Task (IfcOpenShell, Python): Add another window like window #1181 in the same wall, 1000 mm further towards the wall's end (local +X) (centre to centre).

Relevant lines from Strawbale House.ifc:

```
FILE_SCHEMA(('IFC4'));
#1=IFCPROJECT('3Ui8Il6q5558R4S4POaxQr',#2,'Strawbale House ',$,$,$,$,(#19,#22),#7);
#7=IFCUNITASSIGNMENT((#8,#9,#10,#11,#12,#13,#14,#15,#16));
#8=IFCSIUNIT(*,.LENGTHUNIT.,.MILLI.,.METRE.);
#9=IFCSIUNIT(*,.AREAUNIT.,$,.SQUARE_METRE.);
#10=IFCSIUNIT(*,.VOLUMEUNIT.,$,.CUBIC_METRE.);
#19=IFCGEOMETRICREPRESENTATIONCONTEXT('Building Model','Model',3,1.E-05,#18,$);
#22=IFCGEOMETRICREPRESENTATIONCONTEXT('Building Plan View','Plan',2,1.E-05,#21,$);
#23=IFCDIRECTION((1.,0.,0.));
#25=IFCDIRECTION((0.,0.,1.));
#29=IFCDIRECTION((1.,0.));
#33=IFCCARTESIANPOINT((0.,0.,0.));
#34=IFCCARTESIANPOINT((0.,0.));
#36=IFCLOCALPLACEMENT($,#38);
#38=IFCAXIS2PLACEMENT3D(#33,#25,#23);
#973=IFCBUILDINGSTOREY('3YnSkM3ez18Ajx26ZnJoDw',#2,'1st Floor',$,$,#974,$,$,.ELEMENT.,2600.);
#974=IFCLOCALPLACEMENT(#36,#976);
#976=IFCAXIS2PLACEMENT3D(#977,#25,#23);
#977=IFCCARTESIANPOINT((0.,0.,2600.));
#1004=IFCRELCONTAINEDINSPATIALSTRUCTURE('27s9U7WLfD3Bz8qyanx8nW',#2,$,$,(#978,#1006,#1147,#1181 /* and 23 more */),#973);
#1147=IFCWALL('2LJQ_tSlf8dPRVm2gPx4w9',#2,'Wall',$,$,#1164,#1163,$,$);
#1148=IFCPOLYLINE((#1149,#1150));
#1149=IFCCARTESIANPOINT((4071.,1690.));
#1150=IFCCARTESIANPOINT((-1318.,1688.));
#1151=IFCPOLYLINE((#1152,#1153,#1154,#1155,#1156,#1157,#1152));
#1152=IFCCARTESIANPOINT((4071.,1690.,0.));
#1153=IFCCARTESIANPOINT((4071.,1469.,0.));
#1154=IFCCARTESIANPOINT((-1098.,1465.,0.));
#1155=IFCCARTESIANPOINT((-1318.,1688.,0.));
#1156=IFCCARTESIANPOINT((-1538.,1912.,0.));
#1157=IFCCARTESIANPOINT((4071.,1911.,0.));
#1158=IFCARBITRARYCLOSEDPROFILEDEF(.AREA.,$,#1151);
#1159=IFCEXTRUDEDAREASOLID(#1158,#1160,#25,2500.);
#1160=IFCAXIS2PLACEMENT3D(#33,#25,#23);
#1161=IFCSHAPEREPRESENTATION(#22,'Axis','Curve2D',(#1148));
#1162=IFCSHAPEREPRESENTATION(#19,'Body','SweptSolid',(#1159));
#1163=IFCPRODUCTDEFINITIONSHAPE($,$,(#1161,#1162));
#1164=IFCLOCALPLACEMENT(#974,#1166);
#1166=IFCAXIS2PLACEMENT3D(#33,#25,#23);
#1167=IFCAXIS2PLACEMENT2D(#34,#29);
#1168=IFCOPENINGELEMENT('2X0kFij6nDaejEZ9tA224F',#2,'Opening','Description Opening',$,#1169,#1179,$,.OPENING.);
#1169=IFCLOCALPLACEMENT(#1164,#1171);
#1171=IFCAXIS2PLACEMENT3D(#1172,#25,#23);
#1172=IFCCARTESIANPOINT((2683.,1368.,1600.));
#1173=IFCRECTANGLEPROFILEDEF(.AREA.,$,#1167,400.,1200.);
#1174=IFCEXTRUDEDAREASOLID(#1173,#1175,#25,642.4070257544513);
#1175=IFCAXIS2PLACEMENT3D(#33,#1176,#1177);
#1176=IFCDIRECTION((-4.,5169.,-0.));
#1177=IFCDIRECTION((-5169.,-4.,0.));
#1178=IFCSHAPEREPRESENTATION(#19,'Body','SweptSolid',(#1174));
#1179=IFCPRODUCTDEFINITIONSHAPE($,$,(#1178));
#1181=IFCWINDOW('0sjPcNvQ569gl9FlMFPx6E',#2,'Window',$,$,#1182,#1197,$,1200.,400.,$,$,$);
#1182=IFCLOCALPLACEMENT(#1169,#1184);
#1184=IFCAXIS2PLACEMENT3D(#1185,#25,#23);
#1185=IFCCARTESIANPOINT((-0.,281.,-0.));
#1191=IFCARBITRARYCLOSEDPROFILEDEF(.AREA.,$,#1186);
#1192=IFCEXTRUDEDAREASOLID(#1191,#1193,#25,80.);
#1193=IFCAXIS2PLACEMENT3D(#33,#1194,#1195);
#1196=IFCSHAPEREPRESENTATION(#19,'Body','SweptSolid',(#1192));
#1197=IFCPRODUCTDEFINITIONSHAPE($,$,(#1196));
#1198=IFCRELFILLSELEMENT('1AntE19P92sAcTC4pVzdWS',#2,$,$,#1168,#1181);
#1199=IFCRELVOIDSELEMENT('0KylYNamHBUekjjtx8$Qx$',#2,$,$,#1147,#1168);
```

```python
import ifcopenshell
import ifcopenshell.api.feature
import ifcopenshell.api.geometry
import ifcopenshell.api.root
import ifcopenshell.geom
import ifcopenshell.util.element
import ifcopenshell.util.placement
import ifcopenshell.util.shape
import ifcopenshell.util.unit

model = ifcopenshell.open("Strawbale House.ifc")
unit_scale = ifcopenshell.util.unit.calculate_unit_scale(model)
settings = ifcopenshell.geom.settings()


def volume(element):
    """Net volume in cubic metres, openings subtracted."""
    shape = ifcopenshell.geom.create_shape(settings, element)
    return ifcopenshell.util.shape.get_volume(shape.geometry)


window = model.by_guid("0sjPcNvQ569gl9FlMFPx6E")
opening = window.FillsVoids[0].RelatingOpeningElement
wall = opening.VoidsElements[0].RelatingBuildingElement
before = volume(wall)
shift = ifcopenshell.util.placement.get_local_placement(wall.ObjectPlacement)[:3, 0] * 1 / unit_scale

# copy_class copies the void relationship, type, container and properties, but no geometry.
new_opening = ifcopenshell.api.root.copy_class(model, product=opening)
new_opening.Representation = ifcopenshell.util.element.copy_deep(
    model, opening.Representation, exclude=["IfcGeometricRepresentationContext", "IfcRepresentationMap"]
)
new_window = ifcopenshell.api.root.copy_class(model, product=window)
new_window.Representation = ifcopenshell.util.element.copy_deep(
    model, window.Representation, exclude=["IfcGeometricRepresentationContext", "IfcRepresentationMap"]
)
ifcopenshell.api.feature.add_filling(model, opening=new_opening, element=new_window)

for old, new in ((opening, new_opening), (window, new_window)):
    matrix = ifcopenshell.util.placement.get_local_placement(old.ObjectPlacement)
    matrix[:3, 3] += shift
    ifcopenshell.api.geometry.edit_object_placement(model, product=new, matrix=matrix, is_si=False)

after = volume(wall)

print(f"wall volume {before:.3f} -> {after:.3f} m3")

model.write("Strawbale House_rev.ifc")
```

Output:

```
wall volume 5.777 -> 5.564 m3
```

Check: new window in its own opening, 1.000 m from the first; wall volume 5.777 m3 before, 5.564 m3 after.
